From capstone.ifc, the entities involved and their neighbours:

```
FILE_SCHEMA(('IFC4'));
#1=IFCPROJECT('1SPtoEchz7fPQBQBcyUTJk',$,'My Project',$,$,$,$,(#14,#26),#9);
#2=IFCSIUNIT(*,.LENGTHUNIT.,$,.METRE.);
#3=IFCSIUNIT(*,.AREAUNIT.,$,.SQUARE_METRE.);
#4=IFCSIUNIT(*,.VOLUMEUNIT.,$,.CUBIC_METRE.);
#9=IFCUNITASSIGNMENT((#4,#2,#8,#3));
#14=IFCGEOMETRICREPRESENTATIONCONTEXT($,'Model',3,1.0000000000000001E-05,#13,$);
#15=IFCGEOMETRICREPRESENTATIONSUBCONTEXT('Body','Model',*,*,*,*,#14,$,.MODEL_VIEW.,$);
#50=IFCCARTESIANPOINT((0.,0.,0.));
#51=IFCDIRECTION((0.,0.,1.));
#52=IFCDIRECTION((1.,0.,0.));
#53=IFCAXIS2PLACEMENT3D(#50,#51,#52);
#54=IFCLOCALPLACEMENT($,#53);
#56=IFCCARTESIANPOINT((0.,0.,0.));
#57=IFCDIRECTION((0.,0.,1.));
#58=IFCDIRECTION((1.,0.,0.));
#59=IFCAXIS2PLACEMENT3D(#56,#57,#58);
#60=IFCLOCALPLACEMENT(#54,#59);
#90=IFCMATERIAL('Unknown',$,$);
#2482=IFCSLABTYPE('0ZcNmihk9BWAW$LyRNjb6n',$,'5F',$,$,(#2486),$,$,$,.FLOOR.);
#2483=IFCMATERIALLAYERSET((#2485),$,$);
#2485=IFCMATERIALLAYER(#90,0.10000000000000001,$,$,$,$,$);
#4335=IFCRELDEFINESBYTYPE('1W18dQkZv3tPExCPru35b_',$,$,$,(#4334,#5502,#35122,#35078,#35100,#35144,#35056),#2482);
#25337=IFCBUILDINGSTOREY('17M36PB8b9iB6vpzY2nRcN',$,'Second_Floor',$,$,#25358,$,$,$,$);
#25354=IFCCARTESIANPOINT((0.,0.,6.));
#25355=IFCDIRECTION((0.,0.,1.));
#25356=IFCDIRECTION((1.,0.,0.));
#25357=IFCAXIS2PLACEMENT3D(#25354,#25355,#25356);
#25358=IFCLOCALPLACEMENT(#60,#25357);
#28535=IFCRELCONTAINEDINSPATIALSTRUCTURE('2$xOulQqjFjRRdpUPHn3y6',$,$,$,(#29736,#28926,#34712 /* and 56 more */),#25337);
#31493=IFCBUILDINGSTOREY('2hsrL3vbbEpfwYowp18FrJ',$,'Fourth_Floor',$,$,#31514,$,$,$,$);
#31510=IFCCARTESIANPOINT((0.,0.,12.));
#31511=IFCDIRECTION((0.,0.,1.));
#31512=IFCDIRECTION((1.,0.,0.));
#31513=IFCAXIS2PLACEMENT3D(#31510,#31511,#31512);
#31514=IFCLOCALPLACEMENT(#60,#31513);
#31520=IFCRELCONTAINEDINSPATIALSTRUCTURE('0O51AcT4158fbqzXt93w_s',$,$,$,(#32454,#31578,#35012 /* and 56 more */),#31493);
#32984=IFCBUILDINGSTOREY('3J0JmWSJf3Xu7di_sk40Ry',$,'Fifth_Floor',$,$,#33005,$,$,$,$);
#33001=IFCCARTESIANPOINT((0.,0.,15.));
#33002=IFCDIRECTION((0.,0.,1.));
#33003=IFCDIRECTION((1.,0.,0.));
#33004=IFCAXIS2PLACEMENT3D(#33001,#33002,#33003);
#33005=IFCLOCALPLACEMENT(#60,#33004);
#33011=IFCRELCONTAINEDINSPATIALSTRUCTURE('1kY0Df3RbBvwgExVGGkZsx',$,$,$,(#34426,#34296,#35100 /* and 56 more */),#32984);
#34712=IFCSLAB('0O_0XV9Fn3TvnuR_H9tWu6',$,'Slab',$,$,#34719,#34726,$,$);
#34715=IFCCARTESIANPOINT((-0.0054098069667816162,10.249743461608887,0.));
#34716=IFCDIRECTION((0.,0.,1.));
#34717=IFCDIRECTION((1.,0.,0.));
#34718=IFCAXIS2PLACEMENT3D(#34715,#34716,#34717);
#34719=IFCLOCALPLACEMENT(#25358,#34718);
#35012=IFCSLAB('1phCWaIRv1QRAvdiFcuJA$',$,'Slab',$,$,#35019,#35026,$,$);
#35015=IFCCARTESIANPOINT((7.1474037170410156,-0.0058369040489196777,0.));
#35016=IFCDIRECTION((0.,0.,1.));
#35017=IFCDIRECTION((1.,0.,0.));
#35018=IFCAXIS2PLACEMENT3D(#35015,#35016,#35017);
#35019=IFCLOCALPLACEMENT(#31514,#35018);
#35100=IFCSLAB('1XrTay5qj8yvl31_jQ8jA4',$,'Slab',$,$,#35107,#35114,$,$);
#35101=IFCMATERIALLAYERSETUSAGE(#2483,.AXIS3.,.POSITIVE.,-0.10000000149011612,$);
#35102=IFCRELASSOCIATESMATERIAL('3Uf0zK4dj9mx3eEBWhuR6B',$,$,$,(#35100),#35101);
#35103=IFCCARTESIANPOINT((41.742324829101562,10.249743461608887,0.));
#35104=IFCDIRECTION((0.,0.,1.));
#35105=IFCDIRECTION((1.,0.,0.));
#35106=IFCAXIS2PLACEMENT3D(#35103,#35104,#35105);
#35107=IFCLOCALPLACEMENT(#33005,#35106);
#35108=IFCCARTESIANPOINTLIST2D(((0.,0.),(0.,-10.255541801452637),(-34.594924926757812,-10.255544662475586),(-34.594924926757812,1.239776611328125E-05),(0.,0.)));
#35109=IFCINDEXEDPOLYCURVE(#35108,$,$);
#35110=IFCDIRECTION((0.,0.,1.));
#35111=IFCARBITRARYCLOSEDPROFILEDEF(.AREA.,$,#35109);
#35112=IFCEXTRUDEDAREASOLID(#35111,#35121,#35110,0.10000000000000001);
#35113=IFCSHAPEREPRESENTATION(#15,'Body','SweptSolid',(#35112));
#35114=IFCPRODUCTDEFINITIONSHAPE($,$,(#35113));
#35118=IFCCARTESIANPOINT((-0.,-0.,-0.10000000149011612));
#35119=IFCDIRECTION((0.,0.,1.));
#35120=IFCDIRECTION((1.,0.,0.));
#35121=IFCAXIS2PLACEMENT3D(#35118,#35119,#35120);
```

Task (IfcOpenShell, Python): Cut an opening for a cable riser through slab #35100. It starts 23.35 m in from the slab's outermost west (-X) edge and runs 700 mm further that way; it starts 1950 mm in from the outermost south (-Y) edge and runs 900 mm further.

```python
import numpy as np
import ifcopenshell
import ifcopenshell.api.feature
import ifcopenshell.api.geometry
import ifcopenshell.api.root
import ifcopenshell.geom
import ifcopenshell.util.placement
import ifcopenshell.util.representation
import ifcopenshell.util.shape
import ifcopenshell.util.unit

model = ifcopenshell.open("capstone.ifc")
unit_scale = ifcopenshell.util.unit.calculate_unit_scale(model)
settings = ifcopenshell.geom.settings()


def volume(element):
    """Net volume in cubic metres, openings subtracted."""
    shape = ifcopenshell.geom.create_shape(settings, element)
    return ifcopenshell.util.shape.get_volume(shape.geometry)


slab = model.by_guid("1XrTay5qj8yvl31_jQ8jA4")
before = volume(slab)

# Extent in the slab's own axes, in metres. The edges named are its -X and -Y sides.
slab_shape = ifcopenshell.geom.create_shape(settings, slab)
vertices = ifcopenshell.util.shape.get_vertices(slab_shape.geometry)
x_min, y_min, bottom = vertices.min(axis=0)
top = vertices[:, 2].max()

opening = ifcopenshell.api.root.create_entity(model, ifc_class="IfcOpeningElement", name="Cable riser opening", predefined_type="OPENING")
context = ifcopenshell.util.representation.get_context(model, "Model", "Body", "MODEL_VIEW")
width, depth = 0.7, 0.9
outline = [(0.0, 0.0), (width, 0.0), (width, depth), (0.0, depth), (0.0, 0.0)]
# Overshoot both faces by 50 mm so the cut is clean.
shape = ifcopenshell.api.geometry.add_slab_representation(
    model, context=context, depth=top - bottom + 0.1, polyline=outline
)
ifcopenshell.api.geometry.assign_representation(model, product=opening, representation=shape)

matrix = ifcopenshell.util.placement.get_local_placement(slab.ObjectPlacement)
matrix[:, 3] = matrix @ np.append(np.array([x_min + 23.35, y_min + 1.95, bottom - 0.05]) / unit_scale, 1.0)
ifcopenshell.api.geometry.edit_object_placement(model, product=opening, matrix=matrix, is_si=False)
ifcopenshell.api.feature.add_feature(model, feature=opening, element=slab)

after = volume(slab)

print(f"slab volume {before:.3f} -> {after:.3f} m3")

model.write("capstone_v2.ifc")
```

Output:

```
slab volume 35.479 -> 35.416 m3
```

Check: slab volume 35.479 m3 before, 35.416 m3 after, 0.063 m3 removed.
